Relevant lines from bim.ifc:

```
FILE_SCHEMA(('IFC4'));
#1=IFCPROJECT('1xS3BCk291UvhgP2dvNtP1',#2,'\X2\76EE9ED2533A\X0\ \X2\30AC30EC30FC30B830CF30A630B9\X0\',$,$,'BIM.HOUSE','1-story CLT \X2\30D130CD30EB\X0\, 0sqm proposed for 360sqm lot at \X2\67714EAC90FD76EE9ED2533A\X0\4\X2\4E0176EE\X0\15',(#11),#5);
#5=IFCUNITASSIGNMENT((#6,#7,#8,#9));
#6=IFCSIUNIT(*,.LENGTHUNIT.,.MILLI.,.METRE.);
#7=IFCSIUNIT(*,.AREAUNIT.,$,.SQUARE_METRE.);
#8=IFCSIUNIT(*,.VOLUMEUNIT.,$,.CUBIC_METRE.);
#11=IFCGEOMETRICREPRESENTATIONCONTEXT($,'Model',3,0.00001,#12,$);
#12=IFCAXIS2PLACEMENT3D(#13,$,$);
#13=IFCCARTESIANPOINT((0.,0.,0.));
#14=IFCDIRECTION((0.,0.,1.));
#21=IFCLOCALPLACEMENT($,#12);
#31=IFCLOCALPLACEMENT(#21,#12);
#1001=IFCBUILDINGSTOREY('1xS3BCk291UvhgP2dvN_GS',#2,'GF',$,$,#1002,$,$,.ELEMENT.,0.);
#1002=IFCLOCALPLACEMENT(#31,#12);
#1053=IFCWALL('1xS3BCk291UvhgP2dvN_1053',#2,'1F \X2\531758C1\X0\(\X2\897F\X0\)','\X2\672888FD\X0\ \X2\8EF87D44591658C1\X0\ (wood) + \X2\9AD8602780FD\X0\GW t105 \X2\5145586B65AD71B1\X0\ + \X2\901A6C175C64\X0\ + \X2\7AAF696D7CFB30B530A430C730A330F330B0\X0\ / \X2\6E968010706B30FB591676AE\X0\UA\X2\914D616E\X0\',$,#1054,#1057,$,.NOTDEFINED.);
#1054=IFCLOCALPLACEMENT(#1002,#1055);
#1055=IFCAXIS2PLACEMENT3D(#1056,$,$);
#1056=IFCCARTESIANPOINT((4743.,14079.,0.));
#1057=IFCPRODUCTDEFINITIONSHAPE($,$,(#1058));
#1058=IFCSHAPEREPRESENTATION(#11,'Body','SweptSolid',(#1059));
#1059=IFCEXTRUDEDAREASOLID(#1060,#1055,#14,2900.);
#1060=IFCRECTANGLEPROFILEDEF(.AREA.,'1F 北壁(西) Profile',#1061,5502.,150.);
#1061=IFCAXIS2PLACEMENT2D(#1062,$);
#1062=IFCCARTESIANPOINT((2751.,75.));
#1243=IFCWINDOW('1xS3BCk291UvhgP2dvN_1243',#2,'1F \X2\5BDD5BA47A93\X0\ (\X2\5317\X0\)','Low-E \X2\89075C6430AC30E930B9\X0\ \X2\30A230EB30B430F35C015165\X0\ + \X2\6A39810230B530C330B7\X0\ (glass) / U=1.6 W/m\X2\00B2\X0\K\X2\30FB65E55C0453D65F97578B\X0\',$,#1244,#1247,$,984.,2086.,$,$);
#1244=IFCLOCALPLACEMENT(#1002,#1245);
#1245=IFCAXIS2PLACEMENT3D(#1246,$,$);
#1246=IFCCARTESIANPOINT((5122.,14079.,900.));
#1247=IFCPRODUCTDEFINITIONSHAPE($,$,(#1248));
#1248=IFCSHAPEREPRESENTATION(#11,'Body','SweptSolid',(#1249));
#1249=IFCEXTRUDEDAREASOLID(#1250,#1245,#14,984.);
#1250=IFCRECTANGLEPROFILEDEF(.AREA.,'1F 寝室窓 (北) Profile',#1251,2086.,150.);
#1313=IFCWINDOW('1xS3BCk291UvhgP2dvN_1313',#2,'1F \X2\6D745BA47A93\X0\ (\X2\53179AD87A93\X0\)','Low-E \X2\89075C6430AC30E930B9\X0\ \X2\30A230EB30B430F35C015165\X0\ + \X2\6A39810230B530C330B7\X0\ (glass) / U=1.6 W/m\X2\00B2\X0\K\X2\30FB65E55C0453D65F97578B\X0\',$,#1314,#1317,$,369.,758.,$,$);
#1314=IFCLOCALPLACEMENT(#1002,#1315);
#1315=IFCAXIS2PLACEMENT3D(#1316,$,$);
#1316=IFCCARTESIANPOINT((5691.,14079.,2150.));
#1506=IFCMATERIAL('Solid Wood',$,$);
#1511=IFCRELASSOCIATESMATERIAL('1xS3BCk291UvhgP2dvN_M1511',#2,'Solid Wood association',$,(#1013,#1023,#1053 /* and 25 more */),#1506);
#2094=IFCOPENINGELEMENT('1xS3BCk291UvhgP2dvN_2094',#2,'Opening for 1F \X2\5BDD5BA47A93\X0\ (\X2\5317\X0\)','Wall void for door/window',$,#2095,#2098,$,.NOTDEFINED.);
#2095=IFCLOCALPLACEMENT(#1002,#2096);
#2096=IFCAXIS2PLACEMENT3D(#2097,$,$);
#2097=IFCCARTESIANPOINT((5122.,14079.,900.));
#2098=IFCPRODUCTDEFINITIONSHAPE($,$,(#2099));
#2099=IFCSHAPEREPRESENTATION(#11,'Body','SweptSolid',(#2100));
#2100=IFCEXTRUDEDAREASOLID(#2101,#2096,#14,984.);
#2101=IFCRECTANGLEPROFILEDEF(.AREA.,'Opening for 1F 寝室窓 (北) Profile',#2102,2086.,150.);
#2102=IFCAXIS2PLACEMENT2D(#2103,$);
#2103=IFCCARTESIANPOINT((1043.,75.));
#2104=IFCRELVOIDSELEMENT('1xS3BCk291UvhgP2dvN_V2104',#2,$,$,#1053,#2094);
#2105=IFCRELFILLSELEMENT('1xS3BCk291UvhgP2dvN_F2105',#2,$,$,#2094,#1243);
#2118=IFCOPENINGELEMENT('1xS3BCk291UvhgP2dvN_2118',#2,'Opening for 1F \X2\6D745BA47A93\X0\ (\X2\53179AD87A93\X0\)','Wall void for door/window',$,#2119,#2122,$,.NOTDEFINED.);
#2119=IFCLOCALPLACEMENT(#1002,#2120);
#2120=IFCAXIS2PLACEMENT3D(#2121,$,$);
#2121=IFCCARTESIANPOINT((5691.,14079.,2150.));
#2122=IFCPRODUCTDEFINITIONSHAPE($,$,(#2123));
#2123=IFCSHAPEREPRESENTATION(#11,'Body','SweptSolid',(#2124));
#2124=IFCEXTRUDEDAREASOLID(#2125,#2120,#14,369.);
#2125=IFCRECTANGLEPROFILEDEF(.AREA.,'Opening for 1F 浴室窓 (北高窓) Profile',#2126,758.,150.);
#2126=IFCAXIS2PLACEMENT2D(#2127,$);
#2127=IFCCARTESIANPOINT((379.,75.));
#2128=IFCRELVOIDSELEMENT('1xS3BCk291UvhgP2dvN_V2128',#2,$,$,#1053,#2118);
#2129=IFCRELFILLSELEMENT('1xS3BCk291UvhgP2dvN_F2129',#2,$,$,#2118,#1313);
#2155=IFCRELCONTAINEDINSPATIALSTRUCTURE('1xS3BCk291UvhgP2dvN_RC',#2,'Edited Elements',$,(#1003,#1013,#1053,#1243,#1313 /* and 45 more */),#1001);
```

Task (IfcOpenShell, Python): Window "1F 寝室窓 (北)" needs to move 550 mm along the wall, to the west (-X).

```python
import ifcopenshell
import ifcopenshell.api.geometry
import ifcopenshell.util.placement
import ifcopenshell.util.unit

model = ifcopenshell.open("bim.ifc")
unit_scale = ifcopenshell.util.unit.calculate_unit_scale(model)

window = model.by_guid("1xS3BCk291UvhgP2dvN_1243")
opening = window.FillsVoids[0].RelatingOpeningElement
wall = opening.VoidsElements[0].RelatingBuildingElement

wall_matrix = ifcopenshell.util.placement.get_local_placement(wall.ObjectPlacement)
shift = wall_matrix[:3, 0] * -0.55 / unit_scale
before = ifcopenshell.util.placement.get_local_placement(window.ObjectPlacement)[:3, 3].copy()

# The window is not placed relative to its opening, so move both.
for product in (opening, window):
    matrix = ifcopenshell.util.placement.get_local_placement(product.ObjectPlacement)
    matrix[:3, 3] += shift
    ifcopenshell.api.geometry.edit_object_placement(model, product=product, matrix=matrix, is_si=False)

after = ifcopenshell.util.placement.get_local_placement(window.ObjectPlacement)[:3, 3]
print("window moved by", (after - before).round(3) + 0.0)

model.write("bim_rev.ifc")
```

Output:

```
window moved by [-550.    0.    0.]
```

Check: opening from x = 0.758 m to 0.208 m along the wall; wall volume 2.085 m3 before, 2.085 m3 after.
